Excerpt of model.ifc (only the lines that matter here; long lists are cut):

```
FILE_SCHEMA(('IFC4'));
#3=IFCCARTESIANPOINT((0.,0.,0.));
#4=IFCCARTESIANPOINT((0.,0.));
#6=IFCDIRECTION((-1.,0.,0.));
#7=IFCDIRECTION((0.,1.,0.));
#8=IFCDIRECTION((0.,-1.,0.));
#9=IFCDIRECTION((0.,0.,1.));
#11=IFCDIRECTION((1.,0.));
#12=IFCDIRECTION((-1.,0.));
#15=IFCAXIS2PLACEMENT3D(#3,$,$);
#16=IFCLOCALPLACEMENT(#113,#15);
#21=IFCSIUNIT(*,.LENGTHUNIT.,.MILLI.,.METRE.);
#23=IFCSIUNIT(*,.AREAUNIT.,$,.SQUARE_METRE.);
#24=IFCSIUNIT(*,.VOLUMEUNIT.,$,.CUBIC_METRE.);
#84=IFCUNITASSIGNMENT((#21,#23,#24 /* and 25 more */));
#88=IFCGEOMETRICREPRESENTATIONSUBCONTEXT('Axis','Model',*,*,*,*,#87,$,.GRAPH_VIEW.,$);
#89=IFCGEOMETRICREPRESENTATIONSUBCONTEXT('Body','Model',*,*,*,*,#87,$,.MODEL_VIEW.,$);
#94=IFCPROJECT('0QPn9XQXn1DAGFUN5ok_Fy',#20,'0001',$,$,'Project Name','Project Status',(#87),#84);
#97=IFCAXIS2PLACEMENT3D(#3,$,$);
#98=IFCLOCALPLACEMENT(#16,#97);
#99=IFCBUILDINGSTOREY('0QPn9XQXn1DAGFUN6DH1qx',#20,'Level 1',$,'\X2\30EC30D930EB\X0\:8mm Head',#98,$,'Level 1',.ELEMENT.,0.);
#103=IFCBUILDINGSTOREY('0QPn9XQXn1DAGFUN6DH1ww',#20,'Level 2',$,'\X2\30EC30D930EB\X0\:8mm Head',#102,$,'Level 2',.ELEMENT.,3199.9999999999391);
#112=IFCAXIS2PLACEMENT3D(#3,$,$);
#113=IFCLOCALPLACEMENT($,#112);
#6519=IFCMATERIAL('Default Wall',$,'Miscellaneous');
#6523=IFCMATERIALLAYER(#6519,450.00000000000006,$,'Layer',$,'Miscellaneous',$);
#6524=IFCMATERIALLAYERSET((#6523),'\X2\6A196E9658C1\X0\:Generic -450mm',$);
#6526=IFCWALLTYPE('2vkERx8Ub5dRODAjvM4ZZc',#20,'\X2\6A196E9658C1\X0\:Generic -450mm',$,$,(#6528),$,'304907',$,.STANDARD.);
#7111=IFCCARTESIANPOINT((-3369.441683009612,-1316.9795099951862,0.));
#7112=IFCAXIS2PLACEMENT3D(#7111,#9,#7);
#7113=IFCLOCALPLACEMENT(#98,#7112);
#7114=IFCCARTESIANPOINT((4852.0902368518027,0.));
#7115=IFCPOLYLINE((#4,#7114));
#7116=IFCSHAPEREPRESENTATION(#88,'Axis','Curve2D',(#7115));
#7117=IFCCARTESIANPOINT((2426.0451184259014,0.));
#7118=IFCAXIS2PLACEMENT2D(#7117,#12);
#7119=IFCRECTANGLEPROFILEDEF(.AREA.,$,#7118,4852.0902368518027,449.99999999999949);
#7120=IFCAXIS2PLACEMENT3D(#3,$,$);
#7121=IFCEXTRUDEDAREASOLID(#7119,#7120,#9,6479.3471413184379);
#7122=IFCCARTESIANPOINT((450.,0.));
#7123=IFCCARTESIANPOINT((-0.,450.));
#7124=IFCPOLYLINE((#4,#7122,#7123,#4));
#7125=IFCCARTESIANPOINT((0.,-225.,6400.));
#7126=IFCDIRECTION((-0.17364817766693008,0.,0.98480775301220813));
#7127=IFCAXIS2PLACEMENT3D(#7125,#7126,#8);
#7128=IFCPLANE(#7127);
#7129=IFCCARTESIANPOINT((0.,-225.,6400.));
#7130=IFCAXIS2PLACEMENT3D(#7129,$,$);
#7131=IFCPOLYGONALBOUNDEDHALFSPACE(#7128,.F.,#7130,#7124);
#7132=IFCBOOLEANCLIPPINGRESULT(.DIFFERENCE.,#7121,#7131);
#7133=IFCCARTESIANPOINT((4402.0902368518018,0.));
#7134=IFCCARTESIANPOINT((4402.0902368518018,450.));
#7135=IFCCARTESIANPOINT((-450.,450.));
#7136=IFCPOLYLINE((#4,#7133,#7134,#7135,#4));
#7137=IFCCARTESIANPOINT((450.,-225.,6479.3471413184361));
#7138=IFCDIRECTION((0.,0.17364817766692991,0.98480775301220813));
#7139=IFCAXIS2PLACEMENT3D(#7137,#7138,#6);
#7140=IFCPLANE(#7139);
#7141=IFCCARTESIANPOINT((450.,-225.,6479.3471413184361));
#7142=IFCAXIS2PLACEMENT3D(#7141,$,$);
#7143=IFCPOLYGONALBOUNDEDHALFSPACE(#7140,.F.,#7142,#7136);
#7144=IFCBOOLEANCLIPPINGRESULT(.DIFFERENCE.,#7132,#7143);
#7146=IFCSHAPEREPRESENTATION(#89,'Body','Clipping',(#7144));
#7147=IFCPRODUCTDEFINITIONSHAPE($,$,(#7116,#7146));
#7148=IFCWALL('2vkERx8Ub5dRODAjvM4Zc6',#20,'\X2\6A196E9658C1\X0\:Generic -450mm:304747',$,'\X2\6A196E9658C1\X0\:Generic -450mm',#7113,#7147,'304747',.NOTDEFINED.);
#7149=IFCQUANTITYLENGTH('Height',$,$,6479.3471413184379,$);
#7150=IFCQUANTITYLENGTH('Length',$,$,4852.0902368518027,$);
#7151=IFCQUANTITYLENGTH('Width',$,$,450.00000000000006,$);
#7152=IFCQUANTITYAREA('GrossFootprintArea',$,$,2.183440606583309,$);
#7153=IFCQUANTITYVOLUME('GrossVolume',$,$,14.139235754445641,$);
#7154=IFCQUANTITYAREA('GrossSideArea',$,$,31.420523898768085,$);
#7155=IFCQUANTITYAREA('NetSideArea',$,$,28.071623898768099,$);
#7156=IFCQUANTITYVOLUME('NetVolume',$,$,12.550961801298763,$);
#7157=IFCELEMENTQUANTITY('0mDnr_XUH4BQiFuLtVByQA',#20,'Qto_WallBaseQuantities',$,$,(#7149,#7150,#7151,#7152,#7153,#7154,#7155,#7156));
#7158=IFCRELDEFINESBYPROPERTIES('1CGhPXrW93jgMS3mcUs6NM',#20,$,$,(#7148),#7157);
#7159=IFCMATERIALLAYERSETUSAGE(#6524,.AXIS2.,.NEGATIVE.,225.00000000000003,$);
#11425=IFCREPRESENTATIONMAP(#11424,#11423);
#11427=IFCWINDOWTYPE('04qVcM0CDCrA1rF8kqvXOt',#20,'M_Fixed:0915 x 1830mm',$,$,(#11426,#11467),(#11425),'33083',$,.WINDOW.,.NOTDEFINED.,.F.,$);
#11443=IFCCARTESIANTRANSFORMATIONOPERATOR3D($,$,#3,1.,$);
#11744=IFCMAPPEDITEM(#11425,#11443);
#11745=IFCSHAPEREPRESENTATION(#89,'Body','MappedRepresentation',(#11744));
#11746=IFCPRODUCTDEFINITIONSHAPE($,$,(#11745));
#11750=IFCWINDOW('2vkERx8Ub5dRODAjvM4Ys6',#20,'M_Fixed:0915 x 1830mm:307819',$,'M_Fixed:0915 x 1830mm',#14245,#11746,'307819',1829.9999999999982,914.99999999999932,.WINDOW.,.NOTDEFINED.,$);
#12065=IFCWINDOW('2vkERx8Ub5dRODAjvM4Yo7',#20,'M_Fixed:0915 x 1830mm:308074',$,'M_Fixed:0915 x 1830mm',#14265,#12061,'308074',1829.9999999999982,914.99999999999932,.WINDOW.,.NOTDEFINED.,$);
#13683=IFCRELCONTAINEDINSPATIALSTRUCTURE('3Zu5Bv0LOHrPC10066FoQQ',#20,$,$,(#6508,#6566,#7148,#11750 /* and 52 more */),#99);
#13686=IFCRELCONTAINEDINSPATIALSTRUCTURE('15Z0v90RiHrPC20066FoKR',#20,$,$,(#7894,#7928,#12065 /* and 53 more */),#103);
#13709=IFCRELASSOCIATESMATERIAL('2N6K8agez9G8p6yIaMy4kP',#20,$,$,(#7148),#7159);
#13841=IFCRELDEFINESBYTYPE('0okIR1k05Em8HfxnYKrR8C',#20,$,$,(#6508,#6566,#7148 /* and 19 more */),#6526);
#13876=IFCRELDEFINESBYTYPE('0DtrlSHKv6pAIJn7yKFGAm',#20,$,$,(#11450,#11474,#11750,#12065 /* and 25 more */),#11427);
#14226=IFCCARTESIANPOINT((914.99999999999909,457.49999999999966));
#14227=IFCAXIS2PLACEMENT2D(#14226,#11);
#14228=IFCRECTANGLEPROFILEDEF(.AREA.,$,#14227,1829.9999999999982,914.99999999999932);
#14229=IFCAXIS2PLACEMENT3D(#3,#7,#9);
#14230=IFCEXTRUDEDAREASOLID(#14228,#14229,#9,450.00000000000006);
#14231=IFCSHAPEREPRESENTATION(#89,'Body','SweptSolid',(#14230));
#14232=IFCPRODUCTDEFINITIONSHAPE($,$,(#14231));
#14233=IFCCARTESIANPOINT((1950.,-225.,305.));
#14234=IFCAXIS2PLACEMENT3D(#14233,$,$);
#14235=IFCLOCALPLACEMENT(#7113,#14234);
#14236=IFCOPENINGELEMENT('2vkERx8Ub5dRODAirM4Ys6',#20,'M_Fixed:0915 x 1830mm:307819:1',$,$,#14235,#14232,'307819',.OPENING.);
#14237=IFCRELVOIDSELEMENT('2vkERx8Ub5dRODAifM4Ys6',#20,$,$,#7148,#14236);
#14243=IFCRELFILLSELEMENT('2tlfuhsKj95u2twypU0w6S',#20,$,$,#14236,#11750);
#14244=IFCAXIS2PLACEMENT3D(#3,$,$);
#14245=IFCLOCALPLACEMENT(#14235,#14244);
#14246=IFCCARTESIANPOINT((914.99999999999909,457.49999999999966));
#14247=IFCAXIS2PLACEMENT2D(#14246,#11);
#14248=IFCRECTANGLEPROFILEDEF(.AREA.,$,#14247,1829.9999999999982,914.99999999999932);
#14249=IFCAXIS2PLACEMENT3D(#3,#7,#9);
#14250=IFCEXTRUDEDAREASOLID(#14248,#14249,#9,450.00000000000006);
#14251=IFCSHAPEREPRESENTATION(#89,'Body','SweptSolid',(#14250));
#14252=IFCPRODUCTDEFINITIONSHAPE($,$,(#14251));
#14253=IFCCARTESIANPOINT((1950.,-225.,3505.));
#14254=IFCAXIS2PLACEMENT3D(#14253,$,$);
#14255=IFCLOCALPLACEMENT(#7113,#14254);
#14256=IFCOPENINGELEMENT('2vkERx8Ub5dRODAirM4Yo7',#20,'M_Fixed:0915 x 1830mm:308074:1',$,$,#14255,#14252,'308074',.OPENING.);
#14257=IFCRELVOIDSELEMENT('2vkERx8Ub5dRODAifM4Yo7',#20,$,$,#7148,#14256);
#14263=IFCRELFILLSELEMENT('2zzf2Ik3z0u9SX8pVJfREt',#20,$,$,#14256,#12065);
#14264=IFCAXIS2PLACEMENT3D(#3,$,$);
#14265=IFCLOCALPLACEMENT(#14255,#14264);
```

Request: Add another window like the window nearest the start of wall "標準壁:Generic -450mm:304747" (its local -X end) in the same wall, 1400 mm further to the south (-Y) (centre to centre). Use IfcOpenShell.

```python
import ifcopenshell
import ifcopenshell.api.feature
import ifcopenshell.api.geometry
import ifcopenshell.api.pset
import ifcopenshell.api.root
import ifcopenshell.geom
import ifcopenshell.util.element
import ifcopenshell.util.placement
import ifcopenshell.util.shape
import ifcopenshell.util.unit

model = ifcopenshell.open("model.ifc")
unit_scale = ifcopenshell.util.unit.calculate_unit_scale(model)
area_scale = ifcopenshell.util.unit.calculate_unit_scale(model, "AREAUNIT")
volume_scale = ifcopenshell.util.unit.calculate_unit_scale(model, "VOLUMEUNIT")
settings = ifcopenshell.geom.settings()


def volume(element):
    """Net volume in cubic metres, openings subtracted."""
    shape = ifcopenshell.geom.create_shape(settings, element)
    return ifcopenshell.util.shape.get_volume(shape.geometry)


def reuse_history(source, copy):
    """copy_class also copies each property set's owner history, people and application; keep the originals."""
    for rel in copy.IsDefinedBy:
        if rel.is_a("IfcRelDefinesByProperties") and (history := rel.RelatingPropertyDefinition.OwnerHistory):
            rel.RelatingPropertyDefinition.OwnerHistory = source.OwnerHistory
            ifcopenshell.util.element.remove_deep2(model, history)


window = model.by_guid("2vkERx8Ub5dRODAjvM4Ys6")
opening = window.FillsVoids[0].RelatingOpeningElement
wall = opening.VoidsElements[0].RelatingBuildingElement
before = volume(wall)
shift = ifcopenshell.util.placement.get_local_placement(wall.ObjectPlacement)[:3, 0] * -1.4 / unit_scale

# copy_class copies the void relationship, type, container and properties, but no geometry.
new_opening = ifcopenshell.api.root.copy_class(model, product=opening)
new_opening.Representation = ifcopenshell.util.element.copy_deep(
    model, opening.Representation, exclude=["IfcGeometricRepresentationContext", "IfcRepresentationMap"]
)
new_opening.Name = "M_Fixed:0915 x 1830mm"
new_opening.Tag = None
reuse_history(opening, new_opening)
new_window = ifcopenshell.api.root.copy_class(model, product=window)
new_window.Representation = ifcopenshell.util.element.copy_deep(
    model, window.Representation, exclude=["IfcGeometricRepresentationContext", "IfcRepresentationMap"]
)
new_window.Name = "M_Fixed:0915 x 1830mm"
new_window.Tag = None
reuse_history(window, new_window)
ifcopenshell.api.feature.add_filling(model, opening=new_opening, element=new_window)

for old, new in ((opening, new_opening), (window, new_window)):
    matrix = ifcopenshell.util.placement.get_local_placement(old.ObjectPlacement)
    matrix[:3, 3] += shift
    ifcopenshell.api.geometry.edit_object_placement(model, product=new, matrix=matrix, is_si=False)

after = volume(wall)
thickness = 0.45  # wall thickness in metres

# Update the wall's stored quantities.
qto = model.by_id(ifcopenshell.util.element.get_pset(wall, "Qto_WallBaseQuantities", should_inherit=False)["id"])
ifcopenshell.api.pset.edit_qto(model, qto=qto, properties={
    "NetSideArea": after / thickness / area_scale,
    "NetVolume": after / volume_scale,
})

print(f"wall volume {before:.3f} -> {after:.3f} m3")

model.write("model_v2.ifc")
```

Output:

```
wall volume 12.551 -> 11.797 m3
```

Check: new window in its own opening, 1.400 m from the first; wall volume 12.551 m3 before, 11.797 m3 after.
